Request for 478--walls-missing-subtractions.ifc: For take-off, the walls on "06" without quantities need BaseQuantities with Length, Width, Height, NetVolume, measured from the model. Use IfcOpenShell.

First a look at what the model holds.

```python
import ifcopenshell
import ifcopenshell.util.element
import ifcopenshell.util.unit

model = ifcopenshell.open("478--walls-missing-subtractions.ifc")
print(model.schema)
for unit_type in ("LENGTHUNIT", "AREAUNIT", "VOLUMEUNIT"):
    print(unit_type, ifcopenshell.util.unit.calculate_unit_scale(model, unit_type))
storey = next(s for s in model.by_type("IfcBuildingStorey") if s.Name == "06")
walls = [e for e in ifcopenshell.util.element.get_decomposition(storey) if e.is_a("IfcWall")]
for e in sorted(walls, key=lambda e: e.id()):
    print(e.id(), e.is_a(), e.Name, list(ifcopenshell.util.element.get_psets(e, qtos_only=True)), sep=" | ")
```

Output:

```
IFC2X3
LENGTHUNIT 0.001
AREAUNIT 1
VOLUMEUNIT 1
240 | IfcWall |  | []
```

```python
import ifcopenshell
import ifcopenshell.api.pset
import ifcopenshell.geom
import ifcopenshell.util.element
import ifcopenshell.util.shape
import ifcopenshell.util.unit

model = ifcopenshell.open("478--walls-missing-subtractions.ifc")
unit_scale = ifcopenshell.util.unit.calculate_unit_scale(model)
volume_scale = ifcopenshell.util.unit.calculate_unit_scale(model, "VOLUMEUNIT")
settings = ifcopenshell.geom.settings()

storey = next(s for s in model.by_type("IfcBuildingStorey") if s.Name == "06")
walls = [e for e in ifcopenshell.util.element.get_decomposition(storey) if e.is_a("IfcWall")]

for e in sorted(walls, key=lambda e: e.id()):
    if ifcopenshell.util.element.get_psets(e, qtos_only=True, should_inherit=False):
        continue
    # Geometry comes back in metres, in the element's own axes.
    shape = ifcopenshell.geom.create_shape(settings, e)
    values = {
        "Length": ifcopenshell.util.shape.get_x(shape.geometry) / unit_scale,
        "Width": ifcopenshell.util.shape.get_y(shape.geometry) / unit_scale,
        "Height": ifcopenshell.util.shape.get_z(shape.geometry) / unit_scale,
        "NetVolume": ifcopenshell.util.shape.get_volume(shape.geometry) / volume_scale,
    }
    qto = ifcopenshell.api.pset.add_qto(model, product=e, name="BaseQuantities")
    ifcopenshell.api.pset.edit_qto(model, qto=qto, properties=values)
    print(e.id(), {k: round(v, 3) for k, v in values.items()})

model.write("478--walls-missing-subtractions_edited.ifc")
```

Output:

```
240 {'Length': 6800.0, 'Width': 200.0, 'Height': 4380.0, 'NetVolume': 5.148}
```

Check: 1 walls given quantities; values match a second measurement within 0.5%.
